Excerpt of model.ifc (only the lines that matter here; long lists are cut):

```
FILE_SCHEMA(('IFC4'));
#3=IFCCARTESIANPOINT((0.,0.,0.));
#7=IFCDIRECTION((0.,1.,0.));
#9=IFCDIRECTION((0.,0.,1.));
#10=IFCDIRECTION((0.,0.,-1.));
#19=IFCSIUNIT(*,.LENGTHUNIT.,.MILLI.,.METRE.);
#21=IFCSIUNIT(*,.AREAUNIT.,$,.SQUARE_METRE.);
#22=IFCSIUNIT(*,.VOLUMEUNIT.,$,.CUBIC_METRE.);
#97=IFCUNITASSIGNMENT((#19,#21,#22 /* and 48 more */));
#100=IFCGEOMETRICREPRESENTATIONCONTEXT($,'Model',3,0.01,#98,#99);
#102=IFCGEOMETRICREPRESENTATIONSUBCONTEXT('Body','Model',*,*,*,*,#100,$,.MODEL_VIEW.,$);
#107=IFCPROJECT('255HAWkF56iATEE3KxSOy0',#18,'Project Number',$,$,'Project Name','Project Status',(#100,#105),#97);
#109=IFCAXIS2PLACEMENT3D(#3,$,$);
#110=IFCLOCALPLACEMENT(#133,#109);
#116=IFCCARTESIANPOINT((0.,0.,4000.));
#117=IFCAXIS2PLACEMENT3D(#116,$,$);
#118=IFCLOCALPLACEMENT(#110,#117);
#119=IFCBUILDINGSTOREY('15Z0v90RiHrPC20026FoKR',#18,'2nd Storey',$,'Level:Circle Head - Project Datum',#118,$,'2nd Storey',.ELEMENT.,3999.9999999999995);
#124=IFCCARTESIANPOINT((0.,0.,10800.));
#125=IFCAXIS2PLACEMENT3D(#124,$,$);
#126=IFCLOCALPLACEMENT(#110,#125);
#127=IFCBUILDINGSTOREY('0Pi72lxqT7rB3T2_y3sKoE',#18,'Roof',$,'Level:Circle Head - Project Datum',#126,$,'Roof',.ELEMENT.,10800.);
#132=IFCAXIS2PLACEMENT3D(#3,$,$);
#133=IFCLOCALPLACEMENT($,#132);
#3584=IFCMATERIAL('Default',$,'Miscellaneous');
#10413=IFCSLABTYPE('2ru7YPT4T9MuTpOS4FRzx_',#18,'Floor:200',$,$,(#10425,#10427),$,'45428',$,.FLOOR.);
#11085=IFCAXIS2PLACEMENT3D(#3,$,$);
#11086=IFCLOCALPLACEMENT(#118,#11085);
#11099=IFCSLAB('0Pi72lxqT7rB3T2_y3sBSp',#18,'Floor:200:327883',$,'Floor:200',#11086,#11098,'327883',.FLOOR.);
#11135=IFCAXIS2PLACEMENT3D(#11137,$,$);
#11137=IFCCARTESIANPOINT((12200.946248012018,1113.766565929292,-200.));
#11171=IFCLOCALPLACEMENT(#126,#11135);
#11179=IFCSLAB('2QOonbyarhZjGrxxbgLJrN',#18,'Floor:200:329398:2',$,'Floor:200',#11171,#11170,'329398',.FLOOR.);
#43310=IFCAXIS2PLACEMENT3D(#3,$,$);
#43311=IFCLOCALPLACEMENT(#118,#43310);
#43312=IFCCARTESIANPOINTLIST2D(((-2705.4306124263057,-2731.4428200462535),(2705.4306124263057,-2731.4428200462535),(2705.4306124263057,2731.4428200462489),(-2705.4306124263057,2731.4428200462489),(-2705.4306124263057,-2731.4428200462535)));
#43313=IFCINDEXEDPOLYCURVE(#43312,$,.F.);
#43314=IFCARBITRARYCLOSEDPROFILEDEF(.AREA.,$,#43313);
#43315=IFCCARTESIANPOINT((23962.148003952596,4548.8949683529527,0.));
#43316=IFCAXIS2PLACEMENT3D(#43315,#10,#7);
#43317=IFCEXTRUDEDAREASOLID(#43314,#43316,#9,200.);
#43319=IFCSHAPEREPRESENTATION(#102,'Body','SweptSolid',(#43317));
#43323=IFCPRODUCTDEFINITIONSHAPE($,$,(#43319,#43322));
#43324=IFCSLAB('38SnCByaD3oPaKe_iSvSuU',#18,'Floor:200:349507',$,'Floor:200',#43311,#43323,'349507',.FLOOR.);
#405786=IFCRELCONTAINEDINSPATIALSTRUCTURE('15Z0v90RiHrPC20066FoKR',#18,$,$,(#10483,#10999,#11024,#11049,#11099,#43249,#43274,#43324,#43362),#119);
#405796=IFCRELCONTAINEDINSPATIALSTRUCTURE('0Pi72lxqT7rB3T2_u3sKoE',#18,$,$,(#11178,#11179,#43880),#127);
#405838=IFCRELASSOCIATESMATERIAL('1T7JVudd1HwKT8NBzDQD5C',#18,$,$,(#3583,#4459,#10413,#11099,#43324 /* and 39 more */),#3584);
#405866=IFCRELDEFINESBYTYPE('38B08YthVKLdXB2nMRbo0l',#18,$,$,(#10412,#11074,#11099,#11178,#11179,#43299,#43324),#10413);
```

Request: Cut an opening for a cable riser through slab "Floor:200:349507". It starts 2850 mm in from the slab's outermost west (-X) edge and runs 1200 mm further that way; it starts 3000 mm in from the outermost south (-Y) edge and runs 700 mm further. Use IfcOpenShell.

```python
import numpy as np
import ifcopenshell
import ifcopenshell.api.feature
import ifcopenshell.api.geometry
import ifcopenshell.api.root
import ifcopenshell.geom
import ifcopenshell.util.placement
import ifcopenshell.util.representation
import ifcopenshell.util.shape
import ifcopenshell.util.unit

model = ifcopenshell.open("model.ifc")
unit_scale = ifcopenshell.util.unit.calculate_unit_scale(model)
settings = ifcopenshell.geom.settings()


def volume(element):
    """Net volume in cubic metres, openings subtracted."""
    shape = ifcopenshell.geom.create_shape(settings, element)
    return ifcopenshell.util.shape.get_volume(shape.geometry)


slab = model.by_id(43324)
before = volume(slab)

# Extent in the slab's own axes, in metres. The edges named are its -X and -Y sides.
slab_shape = ifcopenshell.geom.create_shape(settings, slab)
vertices = ifcopenshell.util.shape.get_vertices(slab_shape.geometry)
x_min, y_min, bottom = vertices.min(axis=0)
top = vertices[:, 2].max()

opening = ifcopenshell.api.root.create_entity(model, ifc_class="IfcOpeningElement", name="Cable riser opening", predefined_type="OPENING")
context = ifcopenshell.util.representation.get_context(model, "Model", "Body", "MODEL_VIEW")
width, depth = 1.2, 0.7
outline = [(0.0, 0.0), (width, 0.0), (width, depth), (0.0, depth), (0.0, 0.0)]
# Overshoot both faces by 50 mm so the cut is clean.
shape = ifcopenshell.api.geometry.add_slab_representation(
    model, context=context, depth=top - bottom + 0.1, polyline=outline
)
ifcopenshell.api.geometry.assign_representation(model, product=opening, representation=shape)

matrix = ifcopenshell.util.placement.get_local_placement(slab.ObjectPlacement)
matrix[:, 3] = matrix @ np.append(np.array([x_min + 2.85, y_min + 3, bottom - 0.05]) / unit_scale, 1.0)
ifcopenshell.api.geometry.edit_object_placement(model, product=opening, matrix=matrix, is_si=False)
ifcopenshell.api.feature.add_feature(model, feature=opening, element=slab)

after = volume(slab)

print(f"slab volume {before:.3f} -> {after:.3f} m3")

model.write("model_updated.ifc")
```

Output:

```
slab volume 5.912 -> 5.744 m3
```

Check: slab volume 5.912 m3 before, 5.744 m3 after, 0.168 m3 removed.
